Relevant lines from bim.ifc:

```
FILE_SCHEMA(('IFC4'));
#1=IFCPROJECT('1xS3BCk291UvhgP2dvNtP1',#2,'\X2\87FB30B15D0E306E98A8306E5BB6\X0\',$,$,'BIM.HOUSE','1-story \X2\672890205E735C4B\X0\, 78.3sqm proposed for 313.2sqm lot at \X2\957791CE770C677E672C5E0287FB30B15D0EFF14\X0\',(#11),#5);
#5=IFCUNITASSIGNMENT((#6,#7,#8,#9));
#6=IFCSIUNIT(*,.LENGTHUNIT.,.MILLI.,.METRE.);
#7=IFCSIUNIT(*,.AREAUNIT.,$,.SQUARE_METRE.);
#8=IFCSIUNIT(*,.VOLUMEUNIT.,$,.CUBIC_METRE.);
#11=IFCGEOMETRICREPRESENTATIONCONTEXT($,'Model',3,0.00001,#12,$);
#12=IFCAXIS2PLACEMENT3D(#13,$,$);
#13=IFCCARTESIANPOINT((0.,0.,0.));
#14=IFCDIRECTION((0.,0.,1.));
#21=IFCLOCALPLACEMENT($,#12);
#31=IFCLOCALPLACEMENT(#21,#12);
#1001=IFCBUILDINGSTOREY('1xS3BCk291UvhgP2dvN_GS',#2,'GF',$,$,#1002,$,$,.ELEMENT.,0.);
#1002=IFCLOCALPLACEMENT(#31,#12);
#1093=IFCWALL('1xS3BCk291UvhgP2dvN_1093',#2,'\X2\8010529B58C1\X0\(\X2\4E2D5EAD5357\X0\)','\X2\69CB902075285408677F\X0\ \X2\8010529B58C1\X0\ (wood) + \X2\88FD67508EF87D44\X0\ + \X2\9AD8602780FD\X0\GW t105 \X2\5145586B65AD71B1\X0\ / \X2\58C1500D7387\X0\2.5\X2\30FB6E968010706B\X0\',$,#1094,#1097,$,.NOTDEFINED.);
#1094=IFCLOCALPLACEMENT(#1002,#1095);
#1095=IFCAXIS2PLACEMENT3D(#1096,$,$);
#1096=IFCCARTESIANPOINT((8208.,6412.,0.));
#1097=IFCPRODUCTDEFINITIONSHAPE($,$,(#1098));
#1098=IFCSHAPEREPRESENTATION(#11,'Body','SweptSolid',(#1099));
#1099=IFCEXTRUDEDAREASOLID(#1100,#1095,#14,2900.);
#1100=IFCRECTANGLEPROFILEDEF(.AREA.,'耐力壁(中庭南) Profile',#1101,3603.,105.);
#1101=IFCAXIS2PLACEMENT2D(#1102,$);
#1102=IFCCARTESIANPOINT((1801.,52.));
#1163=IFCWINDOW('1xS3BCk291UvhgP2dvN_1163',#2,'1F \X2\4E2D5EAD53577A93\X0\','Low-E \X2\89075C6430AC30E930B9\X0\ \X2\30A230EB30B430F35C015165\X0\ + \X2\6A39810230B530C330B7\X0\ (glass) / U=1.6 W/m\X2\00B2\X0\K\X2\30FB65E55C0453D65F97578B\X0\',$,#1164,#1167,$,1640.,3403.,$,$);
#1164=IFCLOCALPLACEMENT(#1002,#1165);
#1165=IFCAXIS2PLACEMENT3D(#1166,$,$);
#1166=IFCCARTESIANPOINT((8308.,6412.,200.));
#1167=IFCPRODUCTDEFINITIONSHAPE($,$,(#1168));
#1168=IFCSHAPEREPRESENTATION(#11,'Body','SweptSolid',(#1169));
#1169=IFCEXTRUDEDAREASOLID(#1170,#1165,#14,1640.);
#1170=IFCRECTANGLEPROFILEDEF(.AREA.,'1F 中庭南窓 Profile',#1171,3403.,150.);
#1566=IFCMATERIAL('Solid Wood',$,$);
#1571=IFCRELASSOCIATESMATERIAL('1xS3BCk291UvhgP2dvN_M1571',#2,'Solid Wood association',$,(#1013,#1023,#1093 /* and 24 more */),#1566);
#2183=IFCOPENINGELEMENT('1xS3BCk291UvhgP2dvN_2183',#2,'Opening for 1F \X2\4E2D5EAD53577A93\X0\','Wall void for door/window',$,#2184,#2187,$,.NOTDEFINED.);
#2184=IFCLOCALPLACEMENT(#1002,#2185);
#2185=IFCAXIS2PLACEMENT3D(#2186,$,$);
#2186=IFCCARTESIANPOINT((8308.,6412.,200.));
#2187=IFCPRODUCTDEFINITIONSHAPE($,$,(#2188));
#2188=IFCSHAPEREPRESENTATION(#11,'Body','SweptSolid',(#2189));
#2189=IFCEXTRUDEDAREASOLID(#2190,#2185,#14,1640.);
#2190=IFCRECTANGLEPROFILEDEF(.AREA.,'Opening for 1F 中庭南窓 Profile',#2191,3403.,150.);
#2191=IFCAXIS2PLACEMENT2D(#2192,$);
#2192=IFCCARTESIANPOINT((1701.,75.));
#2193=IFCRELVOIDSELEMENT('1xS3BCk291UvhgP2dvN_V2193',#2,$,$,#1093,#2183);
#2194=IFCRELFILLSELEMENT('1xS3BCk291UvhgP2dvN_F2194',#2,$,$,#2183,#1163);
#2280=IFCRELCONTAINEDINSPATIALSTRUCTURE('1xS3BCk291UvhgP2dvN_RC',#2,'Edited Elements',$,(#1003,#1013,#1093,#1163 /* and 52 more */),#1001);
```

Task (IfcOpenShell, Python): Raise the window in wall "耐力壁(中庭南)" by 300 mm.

```python
import numpy as np
import ifcopenshell
import ifcopenshell.api.geometry
import ifcopenshell.util.placement
import ifcopenshell.util.unit

model = ifcopenshell.open("bim.ifc")
unit_scale = ifcopenshell.util.unit.calculate_unit_scale(model)

window = model.by_id(1163)
opening = window.FillsVoids[0].RelatingOpeningElement
dz = 0.3 / unit_scale

shift = np.array([0.0, 0.0, dz])
# The window is not placed relative to its opening, so move both.
for product in (opening, window):
    matrix = ifcopenshell.util.placement.get_local_placement(product.ObjectPlacement)
    matrix[:3, 3] += shift
    ifcopenshell.api.geometry.edit_object_placement(model, product=product, matrix=matrix, is_si=False)

print(f"moved by {dz * unit_scale:+.3f} m")

model.write("bim_rev.ifc")
```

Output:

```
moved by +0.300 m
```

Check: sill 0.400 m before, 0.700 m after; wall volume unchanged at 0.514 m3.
